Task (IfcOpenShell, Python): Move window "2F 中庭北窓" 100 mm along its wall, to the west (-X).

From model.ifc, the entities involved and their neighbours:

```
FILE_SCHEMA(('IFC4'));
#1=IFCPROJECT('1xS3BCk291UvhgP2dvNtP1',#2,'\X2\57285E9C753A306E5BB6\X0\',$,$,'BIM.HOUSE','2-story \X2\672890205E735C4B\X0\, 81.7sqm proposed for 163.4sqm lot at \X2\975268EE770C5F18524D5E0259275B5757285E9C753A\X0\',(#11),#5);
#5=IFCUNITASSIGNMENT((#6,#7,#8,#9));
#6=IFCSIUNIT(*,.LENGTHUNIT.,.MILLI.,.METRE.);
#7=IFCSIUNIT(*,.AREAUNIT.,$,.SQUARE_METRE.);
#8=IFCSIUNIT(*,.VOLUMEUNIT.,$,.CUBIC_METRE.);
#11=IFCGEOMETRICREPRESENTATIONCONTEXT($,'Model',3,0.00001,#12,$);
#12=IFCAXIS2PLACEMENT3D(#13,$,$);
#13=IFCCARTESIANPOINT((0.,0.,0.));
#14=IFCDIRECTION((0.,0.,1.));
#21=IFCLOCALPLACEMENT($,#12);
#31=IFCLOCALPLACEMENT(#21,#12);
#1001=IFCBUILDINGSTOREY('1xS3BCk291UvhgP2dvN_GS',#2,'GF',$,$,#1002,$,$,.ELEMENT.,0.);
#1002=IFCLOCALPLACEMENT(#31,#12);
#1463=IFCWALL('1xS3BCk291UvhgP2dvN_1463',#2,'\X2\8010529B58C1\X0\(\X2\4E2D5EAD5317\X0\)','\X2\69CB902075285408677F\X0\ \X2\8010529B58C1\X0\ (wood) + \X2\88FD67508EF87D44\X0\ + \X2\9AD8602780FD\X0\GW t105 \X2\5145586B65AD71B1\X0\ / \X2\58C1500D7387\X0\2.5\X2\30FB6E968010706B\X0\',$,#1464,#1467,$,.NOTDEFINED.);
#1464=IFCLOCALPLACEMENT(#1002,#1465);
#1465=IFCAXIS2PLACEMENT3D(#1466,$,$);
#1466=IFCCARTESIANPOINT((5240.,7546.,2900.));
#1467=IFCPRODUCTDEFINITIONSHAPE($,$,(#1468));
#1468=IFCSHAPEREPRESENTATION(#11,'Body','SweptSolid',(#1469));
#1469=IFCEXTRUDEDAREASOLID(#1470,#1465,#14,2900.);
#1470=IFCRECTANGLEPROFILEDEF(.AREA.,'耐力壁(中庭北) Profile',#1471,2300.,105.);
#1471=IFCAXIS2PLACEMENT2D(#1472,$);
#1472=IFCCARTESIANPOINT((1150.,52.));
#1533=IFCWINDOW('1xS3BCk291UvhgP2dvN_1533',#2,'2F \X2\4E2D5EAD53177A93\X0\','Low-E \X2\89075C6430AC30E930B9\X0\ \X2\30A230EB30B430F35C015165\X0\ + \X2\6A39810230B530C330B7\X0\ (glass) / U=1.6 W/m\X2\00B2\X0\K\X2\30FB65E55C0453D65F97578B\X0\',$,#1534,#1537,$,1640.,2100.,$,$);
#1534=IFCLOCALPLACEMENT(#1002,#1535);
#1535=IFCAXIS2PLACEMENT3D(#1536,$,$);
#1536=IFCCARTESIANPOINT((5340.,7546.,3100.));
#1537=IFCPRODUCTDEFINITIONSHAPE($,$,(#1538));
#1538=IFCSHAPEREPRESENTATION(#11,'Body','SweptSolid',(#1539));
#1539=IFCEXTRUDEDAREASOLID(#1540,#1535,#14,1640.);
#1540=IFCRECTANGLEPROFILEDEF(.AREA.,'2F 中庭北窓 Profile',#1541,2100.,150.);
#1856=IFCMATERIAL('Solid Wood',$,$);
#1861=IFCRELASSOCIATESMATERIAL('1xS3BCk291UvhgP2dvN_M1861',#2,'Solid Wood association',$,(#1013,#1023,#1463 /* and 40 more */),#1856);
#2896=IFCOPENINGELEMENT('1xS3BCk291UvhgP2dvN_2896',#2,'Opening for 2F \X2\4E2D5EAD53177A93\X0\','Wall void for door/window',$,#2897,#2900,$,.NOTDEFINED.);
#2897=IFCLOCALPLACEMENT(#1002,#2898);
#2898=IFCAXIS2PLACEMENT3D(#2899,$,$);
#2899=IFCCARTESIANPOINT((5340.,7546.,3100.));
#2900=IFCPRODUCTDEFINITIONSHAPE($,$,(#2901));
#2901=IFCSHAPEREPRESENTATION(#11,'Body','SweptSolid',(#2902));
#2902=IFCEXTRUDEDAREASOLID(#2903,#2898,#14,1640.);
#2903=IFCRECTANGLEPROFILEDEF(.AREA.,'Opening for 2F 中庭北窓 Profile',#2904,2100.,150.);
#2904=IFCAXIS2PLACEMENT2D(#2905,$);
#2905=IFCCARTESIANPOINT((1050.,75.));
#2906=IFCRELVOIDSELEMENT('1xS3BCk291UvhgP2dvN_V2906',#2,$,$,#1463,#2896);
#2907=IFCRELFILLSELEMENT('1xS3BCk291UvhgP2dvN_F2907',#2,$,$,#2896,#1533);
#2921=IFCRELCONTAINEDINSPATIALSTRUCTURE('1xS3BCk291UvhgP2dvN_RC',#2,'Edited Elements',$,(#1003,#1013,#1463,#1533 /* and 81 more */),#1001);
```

```python
import ifcopenshell
import ifcopenshell.api.geometry
import ifcopenshell.util.placement
import ifcopenshell.util.unit

model = ifcopenshell.open("model.ifc")
unit_scale = ifcopenshell.util.unit.calculate_unit_scale(model)

window = model.by_id(1533)
opening = window.FillsVoids[0].RelatingOpeningElement
wall = opening.VoidsElements[0].RelatingBuildingElement

wall_matrix = ifcopenshell.util.placement.get_local_placement(wall.ObjectPlacement)
shift = wall_matrix[:3, 0] * -0.1 / unit_scale
before = ifcopenshell.util.placement.get_local_placement(window.ObjectPlacement)[:3, 3].copy()

# The window is not placed relative to its opening, so move both.
for product in (opening, window):
    matrix = ifcopenshell.util.placement.get_local_placement(product.ObjectPlacement)
    matrix[:3, 3] += shift
    ifcopenshell.api.geometry.edit_object_placement(model, product=product, matrix=matrix, is_si=False)

after = ifcopenshell.util.placement.get_local_placement(window.ObjectPlacement)[:3, 3]
print("window moved by", (after - before).round(3) + 0.0)

model.write("model_updated.ifc")
```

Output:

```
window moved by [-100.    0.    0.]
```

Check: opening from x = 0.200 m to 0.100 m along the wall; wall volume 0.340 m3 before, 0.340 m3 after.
